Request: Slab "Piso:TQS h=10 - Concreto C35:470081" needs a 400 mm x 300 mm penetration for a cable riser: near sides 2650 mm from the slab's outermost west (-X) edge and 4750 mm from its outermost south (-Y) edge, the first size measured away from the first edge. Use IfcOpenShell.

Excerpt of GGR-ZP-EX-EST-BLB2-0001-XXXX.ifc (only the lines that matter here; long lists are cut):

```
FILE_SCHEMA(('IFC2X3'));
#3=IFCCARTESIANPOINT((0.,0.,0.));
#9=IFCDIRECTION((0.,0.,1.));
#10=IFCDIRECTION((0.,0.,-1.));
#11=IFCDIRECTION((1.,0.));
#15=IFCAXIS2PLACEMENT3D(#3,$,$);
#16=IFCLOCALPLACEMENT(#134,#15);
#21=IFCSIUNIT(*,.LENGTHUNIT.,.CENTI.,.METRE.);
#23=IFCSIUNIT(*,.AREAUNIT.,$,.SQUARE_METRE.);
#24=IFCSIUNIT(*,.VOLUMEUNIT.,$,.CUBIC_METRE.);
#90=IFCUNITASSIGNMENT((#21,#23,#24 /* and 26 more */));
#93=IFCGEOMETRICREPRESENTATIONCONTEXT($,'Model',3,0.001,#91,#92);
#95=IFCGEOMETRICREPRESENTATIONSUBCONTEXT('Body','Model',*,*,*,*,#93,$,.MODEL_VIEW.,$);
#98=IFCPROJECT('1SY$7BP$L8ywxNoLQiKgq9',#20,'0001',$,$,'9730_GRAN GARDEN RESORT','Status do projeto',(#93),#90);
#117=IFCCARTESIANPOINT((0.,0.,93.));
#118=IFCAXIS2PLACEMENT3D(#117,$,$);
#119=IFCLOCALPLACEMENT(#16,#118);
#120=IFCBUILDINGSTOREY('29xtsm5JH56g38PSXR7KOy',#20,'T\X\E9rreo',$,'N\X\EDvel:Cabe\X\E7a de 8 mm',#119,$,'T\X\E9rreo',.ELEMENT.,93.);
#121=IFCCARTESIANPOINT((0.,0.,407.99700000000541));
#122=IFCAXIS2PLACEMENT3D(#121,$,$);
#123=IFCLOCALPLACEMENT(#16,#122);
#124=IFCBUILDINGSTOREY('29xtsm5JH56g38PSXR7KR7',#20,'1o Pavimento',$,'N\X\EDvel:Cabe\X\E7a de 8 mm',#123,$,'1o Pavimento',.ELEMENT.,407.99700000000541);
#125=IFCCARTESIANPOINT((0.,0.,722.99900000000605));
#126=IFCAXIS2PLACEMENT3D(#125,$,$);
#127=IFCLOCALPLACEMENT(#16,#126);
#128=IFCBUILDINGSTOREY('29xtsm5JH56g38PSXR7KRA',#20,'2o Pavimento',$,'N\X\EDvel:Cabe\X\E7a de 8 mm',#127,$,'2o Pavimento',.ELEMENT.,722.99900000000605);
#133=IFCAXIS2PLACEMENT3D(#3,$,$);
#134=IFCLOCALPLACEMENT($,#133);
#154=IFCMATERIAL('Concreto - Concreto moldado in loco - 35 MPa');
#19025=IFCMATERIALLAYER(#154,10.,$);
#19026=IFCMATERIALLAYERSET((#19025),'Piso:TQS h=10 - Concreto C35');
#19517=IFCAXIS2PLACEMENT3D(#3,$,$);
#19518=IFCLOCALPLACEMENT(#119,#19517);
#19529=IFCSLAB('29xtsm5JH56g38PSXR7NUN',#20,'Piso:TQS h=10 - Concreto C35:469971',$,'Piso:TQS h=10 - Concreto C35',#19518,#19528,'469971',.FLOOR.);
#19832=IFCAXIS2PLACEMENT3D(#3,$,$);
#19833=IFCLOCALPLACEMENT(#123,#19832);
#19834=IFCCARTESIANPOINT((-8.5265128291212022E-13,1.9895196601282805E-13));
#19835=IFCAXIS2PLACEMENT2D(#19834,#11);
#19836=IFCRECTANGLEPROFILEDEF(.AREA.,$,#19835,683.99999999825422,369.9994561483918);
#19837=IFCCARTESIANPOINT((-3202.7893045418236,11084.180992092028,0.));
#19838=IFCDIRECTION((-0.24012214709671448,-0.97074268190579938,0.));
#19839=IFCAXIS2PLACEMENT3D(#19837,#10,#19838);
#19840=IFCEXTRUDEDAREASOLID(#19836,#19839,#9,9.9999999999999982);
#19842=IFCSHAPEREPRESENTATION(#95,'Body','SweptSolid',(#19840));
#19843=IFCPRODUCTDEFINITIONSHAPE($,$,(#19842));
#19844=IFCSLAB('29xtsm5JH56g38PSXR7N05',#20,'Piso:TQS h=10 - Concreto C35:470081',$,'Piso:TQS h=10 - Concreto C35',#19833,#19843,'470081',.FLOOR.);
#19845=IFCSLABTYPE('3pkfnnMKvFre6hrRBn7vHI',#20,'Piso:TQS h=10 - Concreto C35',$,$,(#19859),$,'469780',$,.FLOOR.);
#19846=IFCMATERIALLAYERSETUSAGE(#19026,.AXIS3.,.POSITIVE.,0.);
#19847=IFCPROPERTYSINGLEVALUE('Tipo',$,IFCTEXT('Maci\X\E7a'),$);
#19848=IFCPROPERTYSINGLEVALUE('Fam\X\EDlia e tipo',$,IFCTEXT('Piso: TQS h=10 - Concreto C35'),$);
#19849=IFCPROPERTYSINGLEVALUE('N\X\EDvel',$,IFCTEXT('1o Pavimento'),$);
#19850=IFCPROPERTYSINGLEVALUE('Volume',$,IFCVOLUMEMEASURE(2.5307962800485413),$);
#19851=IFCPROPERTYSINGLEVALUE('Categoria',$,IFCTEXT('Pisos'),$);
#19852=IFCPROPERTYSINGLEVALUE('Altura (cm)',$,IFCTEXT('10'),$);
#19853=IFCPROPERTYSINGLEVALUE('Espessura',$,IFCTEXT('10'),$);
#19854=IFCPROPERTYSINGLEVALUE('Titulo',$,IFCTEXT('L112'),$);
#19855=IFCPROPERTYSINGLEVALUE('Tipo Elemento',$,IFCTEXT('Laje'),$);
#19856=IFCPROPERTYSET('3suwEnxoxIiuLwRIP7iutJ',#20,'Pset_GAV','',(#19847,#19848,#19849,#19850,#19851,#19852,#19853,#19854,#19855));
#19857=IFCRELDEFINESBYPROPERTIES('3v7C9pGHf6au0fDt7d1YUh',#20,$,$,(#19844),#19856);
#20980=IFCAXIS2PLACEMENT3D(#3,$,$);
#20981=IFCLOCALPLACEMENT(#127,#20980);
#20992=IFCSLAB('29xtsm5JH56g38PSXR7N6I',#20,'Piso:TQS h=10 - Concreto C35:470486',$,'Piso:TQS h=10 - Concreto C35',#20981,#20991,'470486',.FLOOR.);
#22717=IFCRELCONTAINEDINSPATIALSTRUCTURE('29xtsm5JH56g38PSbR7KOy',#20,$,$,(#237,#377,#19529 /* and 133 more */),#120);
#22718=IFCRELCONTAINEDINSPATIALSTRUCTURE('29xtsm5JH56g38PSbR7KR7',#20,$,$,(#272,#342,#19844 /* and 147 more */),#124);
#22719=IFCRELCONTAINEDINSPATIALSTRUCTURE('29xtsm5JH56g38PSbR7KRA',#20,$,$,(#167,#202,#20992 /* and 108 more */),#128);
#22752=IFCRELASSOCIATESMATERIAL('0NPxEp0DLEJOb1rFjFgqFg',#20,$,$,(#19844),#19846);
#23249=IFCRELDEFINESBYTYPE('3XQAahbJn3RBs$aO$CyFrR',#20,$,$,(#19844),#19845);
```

```python
import numpy as np
import ifcopenshell
import ifcopenshell.api.feature
import ifcopenshell.api.geometry
import ifcopenshell.api.pset
import ifcopenshell.api.root
import ifcopenshell.geom
import ifcopenshell.util.element
import ifcopenshell.util.placement
import ifcopenshell.util.representation
import ifcopenshell.util.shape
import ifcopenshell.util.unit

model = ifcopenshell.open("GGR-ZP-EX-EST-BLB2-0001-XXXX.ifc")
unit_scale = ifcopenshell.util.unit.calculate_unit_scale(model)
volume_scale = ifcopenshell.util.unit.calculate_unit_scale(model, "VOLUMEUNIT")
settings = ifcopenshell.geom.settings()


def volume(element):
    """Net volume in cubic metres, openings subtracted."""
    shape = ifcopenshell.geom.create_shape(settings, element)
    return ifcopenshell.util.shape.get_volume(shape.geometry)


slab = model.by_guid("29xtsm5JH56g38PSXR7N05")
before = volume(slab)

# Extent in the slab's own axes, in metres. The edges named are its -X and -Y sides.
slab_shape = ifcopenshell.geom.create_shape(settings, slab)
vertices = ifcopenshell.util.shape.get_vertices(slab_shape.geometry)
x_min, y_min, bottom = vertices.min(axis=0)
top = vertices[:, 2].max()

opening = ifcopenshell.api.root.create_entity(model, ifc_class="IfcOpeningElement", name="Cable riser opening")
context = ifcopenshell.util.representation.get_context(model, "Model", "Body", "MODEL_VIEW")
width, depth = 0.4, 0.3
outline = [(0.0, 0.0), (width, 0.0), (width, depth), (0.0, depth), (0.0, 0.0)]
# Overshoot both faces by 50 mm so the cut is clean.
shape = ifcopenshell.api.geometry.add_slab_representation(
    model, context=context, depth=top - bottom + 0.1, polyline=outline
)
ifcopenshell.api.geometry.assign_representation(model, product=opening, representation=shape)

matrix = ifcopenshell.util.placement.get_local_placement(slab.ObjectPlacement)
matrix[:, 3] = matrix @ np.append(np.array([x_min + 2.65, y_min + 4.75, bottom - 0.05]) / unit_scale, 1.0)
ifcopenshell.api.geometry.edit_object_placement(model, product=opening, matrix=matrix, is_si=False)
ifcopenshell.api.feature.add_feature(model, feature=opening, element=slab)

after = volume(slab)

# Update the slab's stored quantities.
pset = model.by_id(ifcopenshell.util.element.get_pset(slab, "Pset_GAV", should_inherit=False)["id"])
ifcopenshell.api.pset.edit_pset(model, pset=pset, properties={
    "Volume": model.create_entity("IfcVolumeMeasure", after / volume_scale),
})

print(f"slab volume {before:.3f} -> {after:.3f} m3")

model.write("GGR-ZP-EX-EST-BLB2-0001-XXXX-out.ifc")
```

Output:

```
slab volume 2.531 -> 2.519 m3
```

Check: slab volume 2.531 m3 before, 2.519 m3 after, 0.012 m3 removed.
